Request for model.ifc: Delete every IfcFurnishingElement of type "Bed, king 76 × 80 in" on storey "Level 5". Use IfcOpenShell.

First a look at what the model holds.

```python
import ifcopenshell
import ifcopenshell.util.element

model = ifcopenshell.open("model.ifc")
print(model.schema)
storey = next(s for s in model.by_type("IfcBuildingStorey") if s.Name == "Level 5")
furniture = [e for e in ifcopenshell.util.element.get_decomposition(storey) if e.is_a("IfcFurnishingElement")]
seen = {}
for e in furniture:
    element_type = ifcopenshell.util.element.get_type(e)
    name = element_type.Name if element_type not in (None, e) else None
    seen[name] = seen.get(name, 0) + 1
for name, count in sorted(seen.items(), key=str):
    print(count, "x", name)
```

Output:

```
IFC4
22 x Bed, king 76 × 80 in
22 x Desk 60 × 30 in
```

```python
import ifcopenshell
import ifcopenshell.api.root
import ifcopenshell.util.element

model = ifcopenshell.open("model.ifc")

storey = next(s for s in model.by_type("IfcBuildingStorey") if s.Name == "Level 5")
furniture = [e for e in ifcopenshell.util.element.get_decomposition(storey) if e.is_a("IfcFurnishingElement")]
targets = [e for e in furniture if (t := ifcopenshell.util.element.get_type(e)) not in (None, e) and t.Name == "Bed, king 76 × 80 in"]

for e in targets:
    ifcopenshell.api.root.remove_product(model, product=e)
print(len(targets), "removed")

model.write("model_edited.ifc")
```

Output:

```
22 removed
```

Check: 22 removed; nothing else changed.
